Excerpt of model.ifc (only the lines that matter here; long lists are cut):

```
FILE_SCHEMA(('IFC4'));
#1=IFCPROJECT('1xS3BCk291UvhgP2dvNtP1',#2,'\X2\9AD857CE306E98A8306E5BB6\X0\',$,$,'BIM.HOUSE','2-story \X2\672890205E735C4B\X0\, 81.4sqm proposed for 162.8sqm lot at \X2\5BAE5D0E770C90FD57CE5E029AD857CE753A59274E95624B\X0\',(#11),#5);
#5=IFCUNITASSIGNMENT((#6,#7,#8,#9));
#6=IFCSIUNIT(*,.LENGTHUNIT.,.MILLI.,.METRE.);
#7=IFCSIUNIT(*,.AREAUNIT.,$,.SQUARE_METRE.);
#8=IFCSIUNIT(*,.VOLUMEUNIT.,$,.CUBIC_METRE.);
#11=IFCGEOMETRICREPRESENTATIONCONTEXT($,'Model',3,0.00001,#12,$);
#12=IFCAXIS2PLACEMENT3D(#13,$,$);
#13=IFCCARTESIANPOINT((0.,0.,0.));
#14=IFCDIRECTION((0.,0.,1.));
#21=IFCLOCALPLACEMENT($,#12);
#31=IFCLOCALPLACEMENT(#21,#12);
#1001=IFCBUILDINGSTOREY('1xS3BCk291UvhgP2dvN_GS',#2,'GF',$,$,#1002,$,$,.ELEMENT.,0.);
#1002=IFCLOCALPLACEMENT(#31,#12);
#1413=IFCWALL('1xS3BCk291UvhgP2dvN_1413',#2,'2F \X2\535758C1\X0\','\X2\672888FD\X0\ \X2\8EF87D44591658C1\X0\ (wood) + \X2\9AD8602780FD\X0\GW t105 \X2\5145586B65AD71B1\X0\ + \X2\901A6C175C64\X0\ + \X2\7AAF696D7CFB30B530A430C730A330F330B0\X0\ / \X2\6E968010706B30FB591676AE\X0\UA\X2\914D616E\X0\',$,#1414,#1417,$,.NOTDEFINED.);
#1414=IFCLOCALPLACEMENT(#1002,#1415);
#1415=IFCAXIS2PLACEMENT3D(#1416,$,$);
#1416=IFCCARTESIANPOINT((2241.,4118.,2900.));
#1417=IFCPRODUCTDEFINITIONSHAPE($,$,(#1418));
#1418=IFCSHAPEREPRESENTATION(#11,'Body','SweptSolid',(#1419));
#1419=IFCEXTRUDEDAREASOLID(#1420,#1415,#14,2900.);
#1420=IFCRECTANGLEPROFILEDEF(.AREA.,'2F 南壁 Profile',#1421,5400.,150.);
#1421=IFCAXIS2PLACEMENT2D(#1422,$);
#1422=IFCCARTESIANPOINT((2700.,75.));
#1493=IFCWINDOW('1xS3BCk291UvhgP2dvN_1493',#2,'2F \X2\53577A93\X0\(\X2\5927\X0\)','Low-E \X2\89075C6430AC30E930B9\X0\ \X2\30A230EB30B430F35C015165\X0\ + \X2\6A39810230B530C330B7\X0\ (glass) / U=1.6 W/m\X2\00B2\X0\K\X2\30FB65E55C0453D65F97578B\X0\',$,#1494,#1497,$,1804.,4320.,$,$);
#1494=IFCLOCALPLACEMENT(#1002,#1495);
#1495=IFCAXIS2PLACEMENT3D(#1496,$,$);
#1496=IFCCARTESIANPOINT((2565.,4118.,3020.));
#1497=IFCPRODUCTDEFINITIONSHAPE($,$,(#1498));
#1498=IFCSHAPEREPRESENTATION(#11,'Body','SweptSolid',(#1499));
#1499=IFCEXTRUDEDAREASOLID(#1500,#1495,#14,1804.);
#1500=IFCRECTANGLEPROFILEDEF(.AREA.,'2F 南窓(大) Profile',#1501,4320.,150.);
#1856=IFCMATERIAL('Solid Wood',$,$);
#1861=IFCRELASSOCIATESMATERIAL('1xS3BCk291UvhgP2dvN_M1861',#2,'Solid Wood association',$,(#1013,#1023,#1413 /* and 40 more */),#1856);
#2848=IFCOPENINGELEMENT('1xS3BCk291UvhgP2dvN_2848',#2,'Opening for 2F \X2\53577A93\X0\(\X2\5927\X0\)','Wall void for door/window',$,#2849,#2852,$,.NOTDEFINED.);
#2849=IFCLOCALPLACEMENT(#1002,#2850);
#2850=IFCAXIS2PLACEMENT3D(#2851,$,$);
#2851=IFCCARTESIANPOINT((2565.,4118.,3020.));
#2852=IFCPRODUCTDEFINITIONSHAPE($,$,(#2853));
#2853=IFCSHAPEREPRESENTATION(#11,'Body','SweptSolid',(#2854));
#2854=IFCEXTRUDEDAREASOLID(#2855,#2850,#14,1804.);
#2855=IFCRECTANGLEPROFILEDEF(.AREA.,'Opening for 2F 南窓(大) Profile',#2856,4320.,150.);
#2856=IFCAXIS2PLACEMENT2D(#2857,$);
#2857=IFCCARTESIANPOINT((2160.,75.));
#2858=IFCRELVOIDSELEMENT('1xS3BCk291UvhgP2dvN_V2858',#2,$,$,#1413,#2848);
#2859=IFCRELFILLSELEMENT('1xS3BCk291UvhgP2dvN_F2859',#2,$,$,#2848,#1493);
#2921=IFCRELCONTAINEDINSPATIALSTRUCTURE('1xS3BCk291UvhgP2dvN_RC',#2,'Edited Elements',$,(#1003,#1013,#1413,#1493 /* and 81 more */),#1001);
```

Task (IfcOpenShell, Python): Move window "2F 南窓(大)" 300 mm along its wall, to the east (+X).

```python
import ifcopenshell
import ifcopenshell.api.geometry
import ifcopenshell.util.placement
import ifcopenshell.util.unit

model = ifcopenshell.open("model.ifc")
unit_scale = ifcopenshell.util.unit.calculate_unit_scale(model)

window = model.by_guid("1xS3BCk291UvhgP2dvN_1493")
opening = window.FillsVoids[0].RelatingOpeningElement
wall = opening.VoidsElements[0].RelatingBuildingElement

wall_matrix = ifcopenshell.util.placement.get_local_placement(wall.ObjectPlacement)
shift = wall_matrix[:3, 0] * 0.3 / unit_scale
before = ifcopenshell.util.placement.get_local_placement(window.ObjectPlacement)[:3, 3].copy()

# The window is not placed relative to its opening, so move both.
for product in (opening, window):
    matrix = ifcopenshell.util.placement.get_local_placement(product.ObjectPlacement)
    matrix[:3, 3] += shift
    ifcopenshell.api.geometry.edit_object_placement(model, product=product, matrix=matrix, is_si=False)

after = ifcopenshell.util.placement.get_local_placement(window.ObjectPlacement)[:3, 3]
print("window moved by", (after - before).round(3) + 0.0)

model.write("model_updated.ifc")
```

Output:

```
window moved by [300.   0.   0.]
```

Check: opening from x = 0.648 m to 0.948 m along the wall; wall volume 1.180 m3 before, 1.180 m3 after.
